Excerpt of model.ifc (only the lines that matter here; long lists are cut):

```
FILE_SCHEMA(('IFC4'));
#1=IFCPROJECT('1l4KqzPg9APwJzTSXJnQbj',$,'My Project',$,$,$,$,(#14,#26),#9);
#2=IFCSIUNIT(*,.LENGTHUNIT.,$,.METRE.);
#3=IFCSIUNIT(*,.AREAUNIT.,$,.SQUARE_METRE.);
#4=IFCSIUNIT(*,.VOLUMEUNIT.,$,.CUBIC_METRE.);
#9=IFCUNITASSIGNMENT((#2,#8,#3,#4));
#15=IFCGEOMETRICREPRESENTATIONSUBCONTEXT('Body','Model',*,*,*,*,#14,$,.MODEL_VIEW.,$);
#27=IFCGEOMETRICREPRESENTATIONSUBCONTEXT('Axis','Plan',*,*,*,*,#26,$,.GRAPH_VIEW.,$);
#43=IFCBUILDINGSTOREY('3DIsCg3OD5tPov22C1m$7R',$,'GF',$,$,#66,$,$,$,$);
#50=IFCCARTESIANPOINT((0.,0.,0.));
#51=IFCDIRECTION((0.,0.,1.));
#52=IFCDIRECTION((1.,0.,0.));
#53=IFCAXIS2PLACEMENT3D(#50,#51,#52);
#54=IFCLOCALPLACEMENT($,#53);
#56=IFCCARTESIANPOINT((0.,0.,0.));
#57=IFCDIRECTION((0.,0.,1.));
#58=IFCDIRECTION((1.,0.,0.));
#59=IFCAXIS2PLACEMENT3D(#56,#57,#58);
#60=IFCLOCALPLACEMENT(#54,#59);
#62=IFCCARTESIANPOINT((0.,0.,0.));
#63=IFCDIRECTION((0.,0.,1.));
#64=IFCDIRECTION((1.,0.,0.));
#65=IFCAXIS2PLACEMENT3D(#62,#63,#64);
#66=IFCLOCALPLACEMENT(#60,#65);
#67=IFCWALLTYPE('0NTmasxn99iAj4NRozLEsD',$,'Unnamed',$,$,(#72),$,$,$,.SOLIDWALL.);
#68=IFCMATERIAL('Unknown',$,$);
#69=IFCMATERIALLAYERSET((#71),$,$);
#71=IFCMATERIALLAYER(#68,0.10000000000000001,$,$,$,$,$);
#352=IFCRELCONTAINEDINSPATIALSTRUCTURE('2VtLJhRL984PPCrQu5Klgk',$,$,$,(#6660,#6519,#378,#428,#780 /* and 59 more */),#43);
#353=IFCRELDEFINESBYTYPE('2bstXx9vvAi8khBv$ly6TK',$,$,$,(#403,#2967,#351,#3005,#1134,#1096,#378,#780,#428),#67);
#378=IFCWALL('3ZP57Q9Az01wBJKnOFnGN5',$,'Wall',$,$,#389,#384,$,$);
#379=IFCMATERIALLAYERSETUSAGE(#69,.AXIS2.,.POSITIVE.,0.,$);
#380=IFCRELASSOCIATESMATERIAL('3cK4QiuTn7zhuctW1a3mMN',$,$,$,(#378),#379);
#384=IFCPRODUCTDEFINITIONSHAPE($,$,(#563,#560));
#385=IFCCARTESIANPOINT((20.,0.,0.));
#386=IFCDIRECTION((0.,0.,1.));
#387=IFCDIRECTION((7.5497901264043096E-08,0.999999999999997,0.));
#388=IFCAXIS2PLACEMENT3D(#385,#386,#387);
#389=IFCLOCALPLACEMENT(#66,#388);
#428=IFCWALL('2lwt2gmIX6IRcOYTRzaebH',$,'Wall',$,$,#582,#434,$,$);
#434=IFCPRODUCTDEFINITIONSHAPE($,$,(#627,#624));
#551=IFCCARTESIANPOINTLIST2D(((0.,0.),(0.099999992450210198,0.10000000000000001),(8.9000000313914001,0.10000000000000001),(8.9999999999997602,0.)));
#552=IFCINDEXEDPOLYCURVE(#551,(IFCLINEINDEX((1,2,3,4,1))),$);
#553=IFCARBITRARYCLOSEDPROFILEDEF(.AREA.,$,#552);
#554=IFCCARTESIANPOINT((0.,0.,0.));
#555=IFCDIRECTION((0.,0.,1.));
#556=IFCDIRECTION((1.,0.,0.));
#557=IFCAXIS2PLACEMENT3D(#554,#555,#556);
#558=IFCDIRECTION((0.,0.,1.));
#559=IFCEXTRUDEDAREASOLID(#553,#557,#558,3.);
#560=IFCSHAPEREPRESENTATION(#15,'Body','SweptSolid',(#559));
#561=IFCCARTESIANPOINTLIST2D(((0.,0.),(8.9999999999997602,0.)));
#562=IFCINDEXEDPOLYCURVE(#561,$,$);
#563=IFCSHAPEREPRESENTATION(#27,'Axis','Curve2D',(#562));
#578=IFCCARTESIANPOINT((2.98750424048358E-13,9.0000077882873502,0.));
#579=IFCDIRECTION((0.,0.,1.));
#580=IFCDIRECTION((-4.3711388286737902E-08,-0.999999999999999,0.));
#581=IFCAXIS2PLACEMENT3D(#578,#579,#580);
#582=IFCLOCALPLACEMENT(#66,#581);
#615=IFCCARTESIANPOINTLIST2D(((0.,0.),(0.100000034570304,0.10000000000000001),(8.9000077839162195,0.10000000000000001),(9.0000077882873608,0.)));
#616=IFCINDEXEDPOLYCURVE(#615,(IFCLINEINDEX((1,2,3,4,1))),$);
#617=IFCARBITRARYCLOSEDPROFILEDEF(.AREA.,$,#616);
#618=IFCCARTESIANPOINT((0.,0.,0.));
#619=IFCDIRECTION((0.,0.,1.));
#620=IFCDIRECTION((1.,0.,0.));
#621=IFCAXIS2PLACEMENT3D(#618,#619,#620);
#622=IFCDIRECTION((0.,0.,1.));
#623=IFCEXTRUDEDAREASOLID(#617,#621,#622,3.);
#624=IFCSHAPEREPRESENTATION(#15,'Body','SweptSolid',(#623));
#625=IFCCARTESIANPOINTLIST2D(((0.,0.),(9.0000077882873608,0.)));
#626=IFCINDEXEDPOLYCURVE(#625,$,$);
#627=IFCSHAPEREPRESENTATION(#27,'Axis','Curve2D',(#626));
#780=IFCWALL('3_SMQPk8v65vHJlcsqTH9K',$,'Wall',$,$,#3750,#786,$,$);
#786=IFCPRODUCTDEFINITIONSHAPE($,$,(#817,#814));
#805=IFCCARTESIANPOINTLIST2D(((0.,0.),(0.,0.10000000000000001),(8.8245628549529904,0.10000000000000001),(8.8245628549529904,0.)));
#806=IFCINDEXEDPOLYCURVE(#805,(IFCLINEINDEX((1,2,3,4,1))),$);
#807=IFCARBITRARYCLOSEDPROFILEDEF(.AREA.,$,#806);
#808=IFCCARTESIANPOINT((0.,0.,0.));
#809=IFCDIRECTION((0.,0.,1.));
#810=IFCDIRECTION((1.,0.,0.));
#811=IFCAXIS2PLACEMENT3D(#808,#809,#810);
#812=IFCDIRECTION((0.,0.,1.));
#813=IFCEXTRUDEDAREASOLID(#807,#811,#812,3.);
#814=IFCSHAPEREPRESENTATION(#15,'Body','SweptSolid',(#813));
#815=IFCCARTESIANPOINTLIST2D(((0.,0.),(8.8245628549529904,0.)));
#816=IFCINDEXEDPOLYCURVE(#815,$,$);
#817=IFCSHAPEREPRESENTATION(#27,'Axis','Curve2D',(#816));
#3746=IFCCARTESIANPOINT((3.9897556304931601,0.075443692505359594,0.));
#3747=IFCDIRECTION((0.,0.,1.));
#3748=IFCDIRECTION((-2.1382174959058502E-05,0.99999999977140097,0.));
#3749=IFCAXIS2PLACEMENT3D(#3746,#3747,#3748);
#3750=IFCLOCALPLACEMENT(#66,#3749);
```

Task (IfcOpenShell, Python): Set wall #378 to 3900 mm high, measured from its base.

```python
import ifcopenshell
import ifcopenshell.geom
import ifcopenshell.util.representation
import ifcopenshell.util.shape

model = ifcopenshell.open("model.ifc")
settings = ifcopenshell.geom.settings()


def volume(element):
    """Net volume in cubic metres, openings subtracted."""
    shape = ifcopenshell.geom.create_shape(settings, element)
    return ifcopenshell.util.shape.get_volume(shape.geometry)


wall = model.by_guid("3ZP57Q9Az01wBJKnOFnGN5")
before = volume(wall)

body = ifcopenshell.util.representation.get_representation(wall, "Model", "Body")
solid = body.Items[0]
old_height = solid.Depth
solid.Depth = 3.9
after = volume(wall)

print(f"height {old_height:g} -> {solid.Depth:g}, volume {before:.3f} -> {after:.3f} m3")

model.write("model-out.ifc")
```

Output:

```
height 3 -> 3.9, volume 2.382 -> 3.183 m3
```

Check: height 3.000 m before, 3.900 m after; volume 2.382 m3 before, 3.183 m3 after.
